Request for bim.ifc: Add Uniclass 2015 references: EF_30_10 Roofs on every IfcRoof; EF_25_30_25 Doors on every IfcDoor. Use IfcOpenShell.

First a look at what the model holds.

```python
import ifcopenshell

model = ifcopenshell.open("bim.ifc")
print(model.schema)
print("classifications:", [c.Name for c in model.by_type("IfcClassification")])
for ifc_class in ("IfcDoor", "IfcRoof", "IfcStair", "IfcWall", "IfcWindow"):
    print(ifc_class, len(model.by_type(ifc_class)))
```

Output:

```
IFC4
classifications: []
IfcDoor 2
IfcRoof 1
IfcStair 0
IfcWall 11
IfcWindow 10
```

```python
import ifcopenshell
import ifcopenshell.api.classification

model = ifcopenshell.open("bim.ifc")

system = ifcopenshell.api.classification.add_classification(model, classification="Uniclass 2015")

codes = {
    "IfcRoof": ("EF_30_10", "Roofs"),
    "IfcDoor": ("EF_25_30_25", "Doors"),
}
for ifc_class, (code, name) in codes.items():
    products = model.by_type(ifc_class)
    ifcopenshell.api.classification.add_reference(
        model, products=products, classification=system, identification=code, name=name
    )
    print(code, len(products))

model.write("bim_updated.ifc")
```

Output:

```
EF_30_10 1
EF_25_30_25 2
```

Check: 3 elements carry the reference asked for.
